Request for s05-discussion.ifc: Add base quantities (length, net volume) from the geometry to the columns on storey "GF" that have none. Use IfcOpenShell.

First a look at what the model holds.

```python
import ifcopenshell
import ifcopenshell.util.element
import ifcopenshell.util.unit

model = ifcopenshell.open("s05-discussion.ifc")
print(model.schema)
for unit_type in ("LENGTHUNIT", "AREAUNIT", "VOLUMEUNIT"):
    print(unit_type, ifcopenshell.util.unit.calculate_unit_scale(model, unit_type))
storey = next(s for s in model.by_type("IfcBuildingStorey") if s.Name == "GF")
columns = [e for e in ifcopenshell.util.element.get_decomposition(storey) if e.is_a("IfcColumn")]
for e in sorted(columns, key=lambda e: e.id()):
    print(e.id(), e.is_a(), e.Name, list(ifcopenshell.util.element.get_psets(e, qtos_only=True)), sep=" | ")
```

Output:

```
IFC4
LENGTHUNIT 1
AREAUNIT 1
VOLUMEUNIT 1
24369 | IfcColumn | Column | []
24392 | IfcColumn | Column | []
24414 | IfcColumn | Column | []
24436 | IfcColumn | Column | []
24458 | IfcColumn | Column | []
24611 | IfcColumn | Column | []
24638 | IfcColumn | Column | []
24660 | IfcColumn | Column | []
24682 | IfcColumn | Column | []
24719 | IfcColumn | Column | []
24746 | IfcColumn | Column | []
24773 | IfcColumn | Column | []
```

```python
import ifcopenshell
import ifcopenshell.api.pset
import ifcopenshell.geom
import ifcopenshell.util.element
import ifcopenshell.util.shape
import ifcopenshell.util.unit

model = ifcopenshell.open("s05-discussion.ifc")
unit_scale = ifcopenshell.util.unit.calculate_unit_scale(model)
volume_scale = ifcopenshell.util.unit.calculate_unit_scale(model, "VOLUMEUNIT")
settings = ifcopenshell.geom.settings()

storey = next(s for s in model.by_type("IfcBuildingStorey") if s.Name == "GF")
columns = [e for e in ifcopenshell.util.element.get_decomposition(storey) if e.is_a("IfcColumn")]

for e in sorted(columns, key=lambda e: e.id()):
    if ifcopenshell.util.element.get_psets(e, qtos_only=True, should_inherit=False):
        continue
    # Geometry comes back in metres, in the element's own axes.
    shape = ifcopenshell.geom.create_shape(settings, e)
    values = {
        "Length": ifcopenshell.util.shape.get_z(shape.geometry) / unit_scale,
        "NetVolume": ifcopenshell.util.shape.get_volume(shape.geometry) / volume_scale,
    }
    qto = ifcopenshell.api.pset.add_qto(model, product=e, name="Qto_ColumnBaseQuantities")
    ifcopenshell.api.pset.edit_qto(model, qto=qto, properties=values)
    print(e.id(), {k: round(v, 3) for k, v in values.items()})

model.write("s05-discussion_updated.ifc")
```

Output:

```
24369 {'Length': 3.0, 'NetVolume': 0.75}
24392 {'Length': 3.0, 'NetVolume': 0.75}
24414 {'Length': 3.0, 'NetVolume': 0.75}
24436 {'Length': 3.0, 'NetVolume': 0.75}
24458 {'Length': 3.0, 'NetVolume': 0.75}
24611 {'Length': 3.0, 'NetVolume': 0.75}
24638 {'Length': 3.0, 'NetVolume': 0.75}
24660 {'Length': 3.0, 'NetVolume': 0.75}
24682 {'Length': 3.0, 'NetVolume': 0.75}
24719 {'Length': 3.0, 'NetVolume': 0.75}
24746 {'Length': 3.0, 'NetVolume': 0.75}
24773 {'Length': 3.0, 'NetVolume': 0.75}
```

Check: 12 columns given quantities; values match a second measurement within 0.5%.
